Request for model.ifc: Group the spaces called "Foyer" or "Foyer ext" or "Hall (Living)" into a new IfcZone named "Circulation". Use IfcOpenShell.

First a look at what the model holds.

```python
import ifcopenshell

model = ifcopenshell.open("model.ifc")
print(model.schema)
seen = {}
for space in model.by_type("IfcSpace"):
    seen[space.LongName] = seen.get(space.LongName, 0) + 1
for name, count in sorted(seen.items(), key=str):
    print(count, "x", name)
print("zones:", [z.Name for z in model.by_type("IfcZone")][:20])
```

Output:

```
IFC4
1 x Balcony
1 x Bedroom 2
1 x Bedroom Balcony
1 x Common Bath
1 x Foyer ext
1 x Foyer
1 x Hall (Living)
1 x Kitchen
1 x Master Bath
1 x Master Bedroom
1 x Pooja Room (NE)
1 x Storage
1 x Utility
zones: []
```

```python
import ifcopenshell
import ifcopenshell.api.group
import ifcopenshell.api.root

model = ifcopenshell.open("model.ifc")

names = {"Foyer", "Foyer ext", "Hall (Living)"}
spaces = [s for s in model.by_type("IfcSpace") if s.LongName in names]

zone = ifcopenshell.api.root.create_entity(model, ifc_class="IfcZone", name="Circulation")
ifcopenshell.api.group.assign_group(model, products=spaces, group=zone)
print(len(spaces), "spaces in", zone.Name)

model.write("model_v2.ifc")
```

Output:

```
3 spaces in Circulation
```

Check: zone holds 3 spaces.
